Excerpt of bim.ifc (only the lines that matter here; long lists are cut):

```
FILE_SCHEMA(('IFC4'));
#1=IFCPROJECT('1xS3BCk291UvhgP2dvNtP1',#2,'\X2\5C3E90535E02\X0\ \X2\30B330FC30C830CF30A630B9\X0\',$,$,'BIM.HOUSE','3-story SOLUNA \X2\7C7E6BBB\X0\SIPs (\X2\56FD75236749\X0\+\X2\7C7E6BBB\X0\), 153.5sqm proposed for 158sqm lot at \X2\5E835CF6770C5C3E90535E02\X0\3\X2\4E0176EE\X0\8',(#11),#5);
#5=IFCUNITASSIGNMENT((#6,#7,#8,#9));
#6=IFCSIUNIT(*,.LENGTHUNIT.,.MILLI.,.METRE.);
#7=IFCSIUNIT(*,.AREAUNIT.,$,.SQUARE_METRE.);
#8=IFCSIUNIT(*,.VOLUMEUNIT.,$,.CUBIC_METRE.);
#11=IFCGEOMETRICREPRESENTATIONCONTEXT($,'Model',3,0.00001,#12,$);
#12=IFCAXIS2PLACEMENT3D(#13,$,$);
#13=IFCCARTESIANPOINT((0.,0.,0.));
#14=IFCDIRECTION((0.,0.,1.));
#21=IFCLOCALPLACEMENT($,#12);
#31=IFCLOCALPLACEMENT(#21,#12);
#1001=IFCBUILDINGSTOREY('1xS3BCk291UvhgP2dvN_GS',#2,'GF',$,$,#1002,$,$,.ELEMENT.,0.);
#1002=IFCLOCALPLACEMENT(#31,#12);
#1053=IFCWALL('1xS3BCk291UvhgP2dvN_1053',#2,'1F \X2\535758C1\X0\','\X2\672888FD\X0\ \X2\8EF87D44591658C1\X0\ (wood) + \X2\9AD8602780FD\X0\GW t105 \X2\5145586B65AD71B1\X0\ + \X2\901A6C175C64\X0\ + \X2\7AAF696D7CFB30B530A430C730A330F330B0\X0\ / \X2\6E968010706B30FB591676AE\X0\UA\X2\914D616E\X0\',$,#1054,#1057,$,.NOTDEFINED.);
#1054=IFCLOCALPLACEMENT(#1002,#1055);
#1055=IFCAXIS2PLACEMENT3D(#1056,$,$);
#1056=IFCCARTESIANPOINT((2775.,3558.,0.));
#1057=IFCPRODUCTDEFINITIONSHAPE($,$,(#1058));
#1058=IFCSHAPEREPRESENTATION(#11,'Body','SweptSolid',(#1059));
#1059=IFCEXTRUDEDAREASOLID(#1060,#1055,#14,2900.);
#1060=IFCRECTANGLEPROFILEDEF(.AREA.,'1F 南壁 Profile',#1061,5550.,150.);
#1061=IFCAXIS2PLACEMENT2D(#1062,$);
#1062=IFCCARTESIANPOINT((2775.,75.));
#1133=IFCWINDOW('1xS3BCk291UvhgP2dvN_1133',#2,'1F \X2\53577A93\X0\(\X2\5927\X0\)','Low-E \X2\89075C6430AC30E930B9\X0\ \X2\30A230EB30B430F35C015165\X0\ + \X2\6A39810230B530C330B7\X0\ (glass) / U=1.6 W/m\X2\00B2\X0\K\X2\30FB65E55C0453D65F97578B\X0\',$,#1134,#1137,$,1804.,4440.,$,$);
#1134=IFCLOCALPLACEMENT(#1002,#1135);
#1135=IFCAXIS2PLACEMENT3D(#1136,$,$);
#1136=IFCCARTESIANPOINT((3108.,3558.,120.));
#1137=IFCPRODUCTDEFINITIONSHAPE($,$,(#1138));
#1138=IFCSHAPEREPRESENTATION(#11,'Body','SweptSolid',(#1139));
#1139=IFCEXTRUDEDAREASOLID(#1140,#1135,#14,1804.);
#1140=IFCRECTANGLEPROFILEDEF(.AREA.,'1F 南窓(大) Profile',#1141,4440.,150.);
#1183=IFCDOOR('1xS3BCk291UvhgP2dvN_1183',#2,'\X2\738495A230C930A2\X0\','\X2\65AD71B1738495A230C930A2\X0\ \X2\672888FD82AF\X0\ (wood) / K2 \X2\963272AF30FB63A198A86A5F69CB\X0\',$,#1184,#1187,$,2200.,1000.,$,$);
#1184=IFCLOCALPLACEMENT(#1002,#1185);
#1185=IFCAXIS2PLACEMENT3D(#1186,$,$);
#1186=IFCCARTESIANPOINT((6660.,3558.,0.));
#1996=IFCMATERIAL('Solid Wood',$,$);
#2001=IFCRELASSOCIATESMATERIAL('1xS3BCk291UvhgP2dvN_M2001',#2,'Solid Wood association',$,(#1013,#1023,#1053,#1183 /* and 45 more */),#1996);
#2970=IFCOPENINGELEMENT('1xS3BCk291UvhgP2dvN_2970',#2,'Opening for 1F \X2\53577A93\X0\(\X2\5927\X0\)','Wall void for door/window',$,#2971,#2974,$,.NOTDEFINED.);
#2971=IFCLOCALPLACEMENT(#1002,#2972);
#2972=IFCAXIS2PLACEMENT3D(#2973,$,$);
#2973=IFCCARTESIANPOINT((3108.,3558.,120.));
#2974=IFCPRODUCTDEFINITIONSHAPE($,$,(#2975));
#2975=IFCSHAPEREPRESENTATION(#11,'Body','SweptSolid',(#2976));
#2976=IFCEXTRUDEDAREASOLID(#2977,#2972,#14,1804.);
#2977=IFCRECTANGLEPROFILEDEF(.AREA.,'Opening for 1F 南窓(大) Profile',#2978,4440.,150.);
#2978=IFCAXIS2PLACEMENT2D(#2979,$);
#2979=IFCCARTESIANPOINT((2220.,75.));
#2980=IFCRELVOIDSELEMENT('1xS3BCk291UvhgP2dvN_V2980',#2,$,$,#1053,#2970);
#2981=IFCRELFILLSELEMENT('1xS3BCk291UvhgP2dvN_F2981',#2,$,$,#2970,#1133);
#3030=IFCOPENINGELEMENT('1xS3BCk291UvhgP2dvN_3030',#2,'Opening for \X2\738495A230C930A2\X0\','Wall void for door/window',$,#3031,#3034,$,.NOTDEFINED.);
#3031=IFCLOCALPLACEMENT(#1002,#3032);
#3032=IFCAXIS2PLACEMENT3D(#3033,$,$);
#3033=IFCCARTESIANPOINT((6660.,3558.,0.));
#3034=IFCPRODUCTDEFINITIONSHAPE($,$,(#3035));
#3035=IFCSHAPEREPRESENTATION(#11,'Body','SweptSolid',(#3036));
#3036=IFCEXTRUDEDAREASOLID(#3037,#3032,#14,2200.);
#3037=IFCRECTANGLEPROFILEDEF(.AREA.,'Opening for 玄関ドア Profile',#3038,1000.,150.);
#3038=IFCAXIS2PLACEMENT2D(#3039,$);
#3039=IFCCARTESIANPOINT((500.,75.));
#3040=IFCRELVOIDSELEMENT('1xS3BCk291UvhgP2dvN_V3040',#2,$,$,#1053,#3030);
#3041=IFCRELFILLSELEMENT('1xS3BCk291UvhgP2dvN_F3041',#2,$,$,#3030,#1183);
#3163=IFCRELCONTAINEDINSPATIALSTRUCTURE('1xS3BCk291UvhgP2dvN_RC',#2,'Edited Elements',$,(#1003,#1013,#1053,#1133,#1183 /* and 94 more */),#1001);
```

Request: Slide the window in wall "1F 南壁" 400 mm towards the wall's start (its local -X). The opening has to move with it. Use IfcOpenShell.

```python
import ifcopenshell
import ifcopenshell.api.geometry
import ifcopenshell.util.placement

model = ifcopenshell.open("bim.ifc")

window = model.by_id(1133)
opening = window.FillsVoids[0].RelatingOpeningElement
wall = opening.VoidsElements[0].RelatingBuildingElement

wall_matrix = ifcopenshell.util.placement.get_local_placement(wall.ObjectPlacement)
shift = wall_matrix[:3, 0] * -400.0
before = ifcopenshell.util.placement.get_local_placement(window.ObjectPlacement)[:3, 3].copy()

# The window is not placed relative to its opening, so move both.
for product in (opening, window):
    matrix = ifcopenshell.util.placement.get_local_placement(product.ObjectPlacement)
    matrix[:3, 3] += shift
    ifcopenshell.api.geometry.edit_object_placement(model, product=product, matrix=matrix, is_si=False)

after = ifcopenshell.util.placement.get_local_placement(window.ObjectPlacement)[:3, 3]
print("window moved by", (after - before).round(3) + 0.0)

model.write("bim_edited.ifc")
```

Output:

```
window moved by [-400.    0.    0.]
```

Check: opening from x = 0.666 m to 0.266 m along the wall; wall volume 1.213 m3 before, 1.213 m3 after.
